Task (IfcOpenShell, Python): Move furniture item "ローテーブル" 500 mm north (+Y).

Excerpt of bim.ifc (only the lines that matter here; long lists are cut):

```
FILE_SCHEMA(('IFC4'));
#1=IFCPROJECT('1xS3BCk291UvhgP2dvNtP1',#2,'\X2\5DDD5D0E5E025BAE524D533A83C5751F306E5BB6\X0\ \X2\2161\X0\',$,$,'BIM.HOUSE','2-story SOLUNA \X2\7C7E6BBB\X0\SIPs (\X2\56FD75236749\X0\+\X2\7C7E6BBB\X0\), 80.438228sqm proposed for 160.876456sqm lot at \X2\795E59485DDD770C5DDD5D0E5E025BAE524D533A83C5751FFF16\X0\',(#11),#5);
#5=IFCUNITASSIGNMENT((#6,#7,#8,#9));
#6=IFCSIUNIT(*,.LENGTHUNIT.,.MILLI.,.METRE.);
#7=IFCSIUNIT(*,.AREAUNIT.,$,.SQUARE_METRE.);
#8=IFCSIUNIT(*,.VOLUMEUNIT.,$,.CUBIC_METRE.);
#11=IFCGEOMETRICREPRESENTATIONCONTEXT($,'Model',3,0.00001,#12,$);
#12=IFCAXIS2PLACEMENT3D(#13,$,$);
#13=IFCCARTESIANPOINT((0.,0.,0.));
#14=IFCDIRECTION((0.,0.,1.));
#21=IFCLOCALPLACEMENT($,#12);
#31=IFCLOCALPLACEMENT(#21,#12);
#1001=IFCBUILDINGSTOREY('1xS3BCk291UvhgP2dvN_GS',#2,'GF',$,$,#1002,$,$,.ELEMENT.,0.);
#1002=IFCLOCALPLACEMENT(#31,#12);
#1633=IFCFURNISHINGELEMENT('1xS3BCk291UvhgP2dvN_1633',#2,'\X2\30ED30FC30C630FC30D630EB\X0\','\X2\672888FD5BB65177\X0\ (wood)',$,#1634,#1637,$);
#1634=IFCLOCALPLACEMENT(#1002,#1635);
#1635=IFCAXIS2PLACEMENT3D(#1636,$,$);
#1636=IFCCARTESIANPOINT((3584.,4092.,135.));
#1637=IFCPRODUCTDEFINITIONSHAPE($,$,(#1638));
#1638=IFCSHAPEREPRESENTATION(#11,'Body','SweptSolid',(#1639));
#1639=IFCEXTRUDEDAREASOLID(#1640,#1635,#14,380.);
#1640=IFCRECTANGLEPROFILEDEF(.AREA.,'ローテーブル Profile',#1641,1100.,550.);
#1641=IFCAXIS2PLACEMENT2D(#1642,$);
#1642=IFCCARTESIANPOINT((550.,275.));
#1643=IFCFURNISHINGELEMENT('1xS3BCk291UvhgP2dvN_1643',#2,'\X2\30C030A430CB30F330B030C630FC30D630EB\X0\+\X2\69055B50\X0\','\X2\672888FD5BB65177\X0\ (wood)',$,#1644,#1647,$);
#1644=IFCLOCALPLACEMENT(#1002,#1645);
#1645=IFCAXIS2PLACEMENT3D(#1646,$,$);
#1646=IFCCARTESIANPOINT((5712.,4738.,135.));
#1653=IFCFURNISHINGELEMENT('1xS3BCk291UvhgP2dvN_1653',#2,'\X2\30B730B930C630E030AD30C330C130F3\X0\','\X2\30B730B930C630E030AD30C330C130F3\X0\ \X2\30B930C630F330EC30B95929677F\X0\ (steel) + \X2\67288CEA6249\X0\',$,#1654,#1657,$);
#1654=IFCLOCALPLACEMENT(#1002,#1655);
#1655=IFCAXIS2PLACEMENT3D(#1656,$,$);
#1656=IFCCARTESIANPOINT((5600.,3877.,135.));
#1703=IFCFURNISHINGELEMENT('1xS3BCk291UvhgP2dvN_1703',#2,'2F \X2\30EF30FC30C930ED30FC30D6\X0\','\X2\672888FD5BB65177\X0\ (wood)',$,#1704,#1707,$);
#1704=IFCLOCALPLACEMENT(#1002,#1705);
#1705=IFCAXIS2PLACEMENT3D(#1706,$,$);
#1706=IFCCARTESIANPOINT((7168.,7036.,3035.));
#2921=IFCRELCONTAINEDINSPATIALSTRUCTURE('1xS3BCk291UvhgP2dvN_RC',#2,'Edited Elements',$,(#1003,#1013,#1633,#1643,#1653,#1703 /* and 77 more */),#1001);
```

```python
import ifcopenshell
import ifcopenshell.api.geometry
import ifcopenshell.util.placement
import ifcopenshell.util.unit

model = ifcopenshell.open("bim.ifc")
unit_scale = ifcopenshell.util.unit.calculate_unit_scale(model)

item = model.by_guid("1xS3BCk291UvhgP2dvN_1633")
matrix = ifcopenshell.util.placement.get_local_placement(item.ObjectPlacement)
matrix[1, 3] += 0.5 / unit_scale
ifcopenshell.api.geometry.edit_object_placement(model, product=item, matrix=matrix, is_si=False)

print(ifcopenshell.util.placement.get_local_placement(item.ObjectPlacement).round(3) + 0.0)

model.write("bim_v2.ifc")
```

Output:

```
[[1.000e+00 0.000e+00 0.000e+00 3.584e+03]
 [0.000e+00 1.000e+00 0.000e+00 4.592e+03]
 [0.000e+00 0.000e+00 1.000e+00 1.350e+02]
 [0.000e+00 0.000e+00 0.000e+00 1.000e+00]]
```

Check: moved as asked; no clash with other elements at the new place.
